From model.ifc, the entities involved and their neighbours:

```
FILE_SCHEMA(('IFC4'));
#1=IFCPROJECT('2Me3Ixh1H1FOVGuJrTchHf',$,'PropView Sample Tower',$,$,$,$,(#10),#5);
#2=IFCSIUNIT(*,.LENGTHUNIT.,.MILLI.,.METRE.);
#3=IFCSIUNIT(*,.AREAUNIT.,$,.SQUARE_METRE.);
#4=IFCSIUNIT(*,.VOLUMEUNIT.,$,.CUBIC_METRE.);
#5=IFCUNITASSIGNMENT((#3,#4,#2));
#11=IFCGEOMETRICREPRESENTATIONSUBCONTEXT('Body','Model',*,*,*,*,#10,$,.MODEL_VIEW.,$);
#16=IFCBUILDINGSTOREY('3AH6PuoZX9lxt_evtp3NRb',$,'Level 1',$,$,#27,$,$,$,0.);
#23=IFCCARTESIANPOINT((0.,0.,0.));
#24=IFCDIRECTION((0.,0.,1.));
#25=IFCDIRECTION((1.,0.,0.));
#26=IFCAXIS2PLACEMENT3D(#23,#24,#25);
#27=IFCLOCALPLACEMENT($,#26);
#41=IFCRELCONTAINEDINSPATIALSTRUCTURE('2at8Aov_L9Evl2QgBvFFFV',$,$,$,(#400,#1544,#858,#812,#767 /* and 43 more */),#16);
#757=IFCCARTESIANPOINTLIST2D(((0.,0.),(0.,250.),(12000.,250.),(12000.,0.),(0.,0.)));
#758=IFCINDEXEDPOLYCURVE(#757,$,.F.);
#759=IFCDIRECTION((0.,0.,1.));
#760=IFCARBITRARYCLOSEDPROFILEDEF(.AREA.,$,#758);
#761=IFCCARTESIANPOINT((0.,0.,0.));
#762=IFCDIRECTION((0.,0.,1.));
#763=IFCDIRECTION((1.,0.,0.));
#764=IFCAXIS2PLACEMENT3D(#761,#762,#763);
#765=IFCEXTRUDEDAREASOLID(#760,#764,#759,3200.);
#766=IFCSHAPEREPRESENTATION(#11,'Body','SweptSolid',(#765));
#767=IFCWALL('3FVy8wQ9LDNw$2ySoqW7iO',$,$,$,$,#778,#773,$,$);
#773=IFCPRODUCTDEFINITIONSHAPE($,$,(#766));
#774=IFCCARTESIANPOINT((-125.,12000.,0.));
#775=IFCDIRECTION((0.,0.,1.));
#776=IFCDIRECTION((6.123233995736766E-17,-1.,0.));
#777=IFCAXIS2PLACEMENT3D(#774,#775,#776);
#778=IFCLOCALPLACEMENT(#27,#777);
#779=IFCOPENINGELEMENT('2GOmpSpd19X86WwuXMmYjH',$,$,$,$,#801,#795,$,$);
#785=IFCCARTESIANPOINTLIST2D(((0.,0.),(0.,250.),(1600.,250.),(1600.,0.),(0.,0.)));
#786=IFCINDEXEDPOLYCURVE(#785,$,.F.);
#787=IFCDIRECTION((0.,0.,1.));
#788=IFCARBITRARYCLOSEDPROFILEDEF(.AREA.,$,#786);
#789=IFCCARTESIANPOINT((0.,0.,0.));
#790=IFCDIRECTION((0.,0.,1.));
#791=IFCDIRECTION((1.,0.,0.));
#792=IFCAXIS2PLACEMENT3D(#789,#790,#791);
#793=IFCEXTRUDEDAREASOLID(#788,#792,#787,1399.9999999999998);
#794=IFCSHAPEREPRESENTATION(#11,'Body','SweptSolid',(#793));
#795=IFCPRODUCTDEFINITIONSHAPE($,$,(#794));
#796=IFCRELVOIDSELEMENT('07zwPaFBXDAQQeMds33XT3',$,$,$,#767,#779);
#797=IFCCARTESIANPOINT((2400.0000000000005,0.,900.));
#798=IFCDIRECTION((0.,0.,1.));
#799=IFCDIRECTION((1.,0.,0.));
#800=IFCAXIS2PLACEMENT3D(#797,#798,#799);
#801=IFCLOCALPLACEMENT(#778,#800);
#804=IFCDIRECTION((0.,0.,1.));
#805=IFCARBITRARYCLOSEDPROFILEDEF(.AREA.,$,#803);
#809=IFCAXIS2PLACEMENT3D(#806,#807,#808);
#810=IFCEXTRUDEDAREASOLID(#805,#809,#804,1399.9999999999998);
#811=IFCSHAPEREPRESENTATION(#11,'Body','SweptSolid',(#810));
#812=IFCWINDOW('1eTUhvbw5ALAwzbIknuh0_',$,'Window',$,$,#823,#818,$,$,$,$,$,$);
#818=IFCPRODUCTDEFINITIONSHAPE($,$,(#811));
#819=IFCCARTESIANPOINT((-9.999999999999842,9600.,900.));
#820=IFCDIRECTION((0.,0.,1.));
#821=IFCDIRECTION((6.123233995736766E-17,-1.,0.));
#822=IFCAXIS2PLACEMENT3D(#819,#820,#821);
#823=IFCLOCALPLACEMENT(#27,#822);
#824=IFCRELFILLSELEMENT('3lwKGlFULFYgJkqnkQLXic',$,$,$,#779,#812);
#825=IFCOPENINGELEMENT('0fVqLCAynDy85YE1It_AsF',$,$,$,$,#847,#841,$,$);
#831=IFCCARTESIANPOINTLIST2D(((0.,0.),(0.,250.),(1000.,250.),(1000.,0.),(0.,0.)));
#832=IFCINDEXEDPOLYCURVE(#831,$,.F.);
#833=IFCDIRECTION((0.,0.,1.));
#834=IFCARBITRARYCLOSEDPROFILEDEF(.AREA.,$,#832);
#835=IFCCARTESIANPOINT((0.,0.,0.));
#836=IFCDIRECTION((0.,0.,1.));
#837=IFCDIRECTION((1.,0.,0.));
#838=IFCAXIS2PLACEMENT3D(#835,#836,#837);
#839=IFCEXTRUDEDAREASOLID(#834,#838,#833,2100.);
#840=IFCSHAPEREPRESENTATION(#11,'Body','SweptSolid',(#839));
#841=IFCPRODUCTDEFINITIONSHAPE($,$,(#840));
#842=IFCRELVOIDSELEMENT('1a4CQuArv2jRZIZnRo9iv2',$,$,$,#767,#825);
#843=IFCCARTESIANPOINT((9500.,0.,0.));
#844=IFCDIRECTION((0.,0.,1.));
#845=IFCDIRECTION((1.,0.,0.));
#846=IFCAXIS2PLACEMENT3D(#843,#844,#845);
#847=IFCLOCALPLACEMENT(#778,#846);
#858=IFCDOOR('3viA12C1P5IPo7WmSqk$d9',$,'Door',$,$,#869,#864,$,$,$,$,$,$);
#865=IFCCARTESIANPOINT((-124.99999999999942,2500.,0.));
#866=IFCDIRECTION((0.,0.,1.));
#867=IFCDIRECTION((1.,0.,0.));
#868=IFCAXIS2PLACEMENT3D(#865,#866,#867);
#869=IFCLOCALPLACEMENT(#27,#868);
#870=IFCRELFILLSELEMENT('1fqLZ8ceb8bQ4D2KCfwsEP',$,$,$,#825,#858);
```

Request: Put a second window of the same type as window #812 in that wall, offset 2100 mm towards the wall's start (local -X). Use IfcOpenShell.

```python
import ifcopenshell
import ifcopenshell.api.feature
import ifcopenshell.api.geometry
import ifcopenshell.api.root
import ifcopenshell.geom
import ifcopenshell.util.element
import ifcopenshell.util.placement
import ifcopenshell.util.shape
import ifcopenshell.util.unit

model = ifcopenshell.open("model.ifc")
unit_scale = ifcopenshell.util.unit.calculate_unit_scale(model)
settings = ifcopenshell.geom.settings()


def volume(element):
    """Net volume in cubic metres, openings subtracted."""
    shape = ifcopenshell.geom.create_shape(settings, element)
    return ifcopenshell.util.shape.get_volume(shape.geometry)


window = model.by_id(812)
opening = window.FillsVoids[0].RelatingOpeningElement
wall = opening.VoidsElements[0].RelatingBuildingElement
before = volume(wall)
shift = ifcopenshell.util.placement.get_local_placement(wall.ObjectPlacement)[:3, 0] * -2.1 / unit_scale

# copy_class copies the void relationship, type, container and properties, but no geometry.
new_opening = ifcopenshell.api.root.copy_class(model, product=opening)
new_opening.Representation = ifcopenshell.util.element.copy_deep(
    model, opening.Representation, exclude=["IfcGeometricRepresentationContext", "IfcRepresentationMap"]
)
new_window = ifcopenshell.api.root.copy_class(model, product=window)
new_window.Representation = ifcopenshell.util.element.copy_deep(
    model, window.Representation, exclude=["IfcGeometricRepresentationContext", "IfcRepresentationMap"]
)
ifcopenshell.api.feature.add_filling(model, opening=new_opening, element=new_window)

for old, new in ((opening, new_opening), (window, new_window)):
    matrix = ifcopenshell.util.placement.get_local_placement(old.ObjectPlacement)
    matrix[:3, 3] += shift
    ifcopenshell.api.geometry.edit_object_placement(model, product=new, matrix=matrix, is_si=False)

after = volume(wall)

print(f"wall volume {before:.3f} -> {after:.3f} m3")

model.write("model_updated.ifc")
```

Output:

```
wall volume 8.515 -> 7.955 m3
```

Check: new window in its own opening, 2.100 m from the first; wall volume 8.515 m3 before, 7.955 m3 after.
